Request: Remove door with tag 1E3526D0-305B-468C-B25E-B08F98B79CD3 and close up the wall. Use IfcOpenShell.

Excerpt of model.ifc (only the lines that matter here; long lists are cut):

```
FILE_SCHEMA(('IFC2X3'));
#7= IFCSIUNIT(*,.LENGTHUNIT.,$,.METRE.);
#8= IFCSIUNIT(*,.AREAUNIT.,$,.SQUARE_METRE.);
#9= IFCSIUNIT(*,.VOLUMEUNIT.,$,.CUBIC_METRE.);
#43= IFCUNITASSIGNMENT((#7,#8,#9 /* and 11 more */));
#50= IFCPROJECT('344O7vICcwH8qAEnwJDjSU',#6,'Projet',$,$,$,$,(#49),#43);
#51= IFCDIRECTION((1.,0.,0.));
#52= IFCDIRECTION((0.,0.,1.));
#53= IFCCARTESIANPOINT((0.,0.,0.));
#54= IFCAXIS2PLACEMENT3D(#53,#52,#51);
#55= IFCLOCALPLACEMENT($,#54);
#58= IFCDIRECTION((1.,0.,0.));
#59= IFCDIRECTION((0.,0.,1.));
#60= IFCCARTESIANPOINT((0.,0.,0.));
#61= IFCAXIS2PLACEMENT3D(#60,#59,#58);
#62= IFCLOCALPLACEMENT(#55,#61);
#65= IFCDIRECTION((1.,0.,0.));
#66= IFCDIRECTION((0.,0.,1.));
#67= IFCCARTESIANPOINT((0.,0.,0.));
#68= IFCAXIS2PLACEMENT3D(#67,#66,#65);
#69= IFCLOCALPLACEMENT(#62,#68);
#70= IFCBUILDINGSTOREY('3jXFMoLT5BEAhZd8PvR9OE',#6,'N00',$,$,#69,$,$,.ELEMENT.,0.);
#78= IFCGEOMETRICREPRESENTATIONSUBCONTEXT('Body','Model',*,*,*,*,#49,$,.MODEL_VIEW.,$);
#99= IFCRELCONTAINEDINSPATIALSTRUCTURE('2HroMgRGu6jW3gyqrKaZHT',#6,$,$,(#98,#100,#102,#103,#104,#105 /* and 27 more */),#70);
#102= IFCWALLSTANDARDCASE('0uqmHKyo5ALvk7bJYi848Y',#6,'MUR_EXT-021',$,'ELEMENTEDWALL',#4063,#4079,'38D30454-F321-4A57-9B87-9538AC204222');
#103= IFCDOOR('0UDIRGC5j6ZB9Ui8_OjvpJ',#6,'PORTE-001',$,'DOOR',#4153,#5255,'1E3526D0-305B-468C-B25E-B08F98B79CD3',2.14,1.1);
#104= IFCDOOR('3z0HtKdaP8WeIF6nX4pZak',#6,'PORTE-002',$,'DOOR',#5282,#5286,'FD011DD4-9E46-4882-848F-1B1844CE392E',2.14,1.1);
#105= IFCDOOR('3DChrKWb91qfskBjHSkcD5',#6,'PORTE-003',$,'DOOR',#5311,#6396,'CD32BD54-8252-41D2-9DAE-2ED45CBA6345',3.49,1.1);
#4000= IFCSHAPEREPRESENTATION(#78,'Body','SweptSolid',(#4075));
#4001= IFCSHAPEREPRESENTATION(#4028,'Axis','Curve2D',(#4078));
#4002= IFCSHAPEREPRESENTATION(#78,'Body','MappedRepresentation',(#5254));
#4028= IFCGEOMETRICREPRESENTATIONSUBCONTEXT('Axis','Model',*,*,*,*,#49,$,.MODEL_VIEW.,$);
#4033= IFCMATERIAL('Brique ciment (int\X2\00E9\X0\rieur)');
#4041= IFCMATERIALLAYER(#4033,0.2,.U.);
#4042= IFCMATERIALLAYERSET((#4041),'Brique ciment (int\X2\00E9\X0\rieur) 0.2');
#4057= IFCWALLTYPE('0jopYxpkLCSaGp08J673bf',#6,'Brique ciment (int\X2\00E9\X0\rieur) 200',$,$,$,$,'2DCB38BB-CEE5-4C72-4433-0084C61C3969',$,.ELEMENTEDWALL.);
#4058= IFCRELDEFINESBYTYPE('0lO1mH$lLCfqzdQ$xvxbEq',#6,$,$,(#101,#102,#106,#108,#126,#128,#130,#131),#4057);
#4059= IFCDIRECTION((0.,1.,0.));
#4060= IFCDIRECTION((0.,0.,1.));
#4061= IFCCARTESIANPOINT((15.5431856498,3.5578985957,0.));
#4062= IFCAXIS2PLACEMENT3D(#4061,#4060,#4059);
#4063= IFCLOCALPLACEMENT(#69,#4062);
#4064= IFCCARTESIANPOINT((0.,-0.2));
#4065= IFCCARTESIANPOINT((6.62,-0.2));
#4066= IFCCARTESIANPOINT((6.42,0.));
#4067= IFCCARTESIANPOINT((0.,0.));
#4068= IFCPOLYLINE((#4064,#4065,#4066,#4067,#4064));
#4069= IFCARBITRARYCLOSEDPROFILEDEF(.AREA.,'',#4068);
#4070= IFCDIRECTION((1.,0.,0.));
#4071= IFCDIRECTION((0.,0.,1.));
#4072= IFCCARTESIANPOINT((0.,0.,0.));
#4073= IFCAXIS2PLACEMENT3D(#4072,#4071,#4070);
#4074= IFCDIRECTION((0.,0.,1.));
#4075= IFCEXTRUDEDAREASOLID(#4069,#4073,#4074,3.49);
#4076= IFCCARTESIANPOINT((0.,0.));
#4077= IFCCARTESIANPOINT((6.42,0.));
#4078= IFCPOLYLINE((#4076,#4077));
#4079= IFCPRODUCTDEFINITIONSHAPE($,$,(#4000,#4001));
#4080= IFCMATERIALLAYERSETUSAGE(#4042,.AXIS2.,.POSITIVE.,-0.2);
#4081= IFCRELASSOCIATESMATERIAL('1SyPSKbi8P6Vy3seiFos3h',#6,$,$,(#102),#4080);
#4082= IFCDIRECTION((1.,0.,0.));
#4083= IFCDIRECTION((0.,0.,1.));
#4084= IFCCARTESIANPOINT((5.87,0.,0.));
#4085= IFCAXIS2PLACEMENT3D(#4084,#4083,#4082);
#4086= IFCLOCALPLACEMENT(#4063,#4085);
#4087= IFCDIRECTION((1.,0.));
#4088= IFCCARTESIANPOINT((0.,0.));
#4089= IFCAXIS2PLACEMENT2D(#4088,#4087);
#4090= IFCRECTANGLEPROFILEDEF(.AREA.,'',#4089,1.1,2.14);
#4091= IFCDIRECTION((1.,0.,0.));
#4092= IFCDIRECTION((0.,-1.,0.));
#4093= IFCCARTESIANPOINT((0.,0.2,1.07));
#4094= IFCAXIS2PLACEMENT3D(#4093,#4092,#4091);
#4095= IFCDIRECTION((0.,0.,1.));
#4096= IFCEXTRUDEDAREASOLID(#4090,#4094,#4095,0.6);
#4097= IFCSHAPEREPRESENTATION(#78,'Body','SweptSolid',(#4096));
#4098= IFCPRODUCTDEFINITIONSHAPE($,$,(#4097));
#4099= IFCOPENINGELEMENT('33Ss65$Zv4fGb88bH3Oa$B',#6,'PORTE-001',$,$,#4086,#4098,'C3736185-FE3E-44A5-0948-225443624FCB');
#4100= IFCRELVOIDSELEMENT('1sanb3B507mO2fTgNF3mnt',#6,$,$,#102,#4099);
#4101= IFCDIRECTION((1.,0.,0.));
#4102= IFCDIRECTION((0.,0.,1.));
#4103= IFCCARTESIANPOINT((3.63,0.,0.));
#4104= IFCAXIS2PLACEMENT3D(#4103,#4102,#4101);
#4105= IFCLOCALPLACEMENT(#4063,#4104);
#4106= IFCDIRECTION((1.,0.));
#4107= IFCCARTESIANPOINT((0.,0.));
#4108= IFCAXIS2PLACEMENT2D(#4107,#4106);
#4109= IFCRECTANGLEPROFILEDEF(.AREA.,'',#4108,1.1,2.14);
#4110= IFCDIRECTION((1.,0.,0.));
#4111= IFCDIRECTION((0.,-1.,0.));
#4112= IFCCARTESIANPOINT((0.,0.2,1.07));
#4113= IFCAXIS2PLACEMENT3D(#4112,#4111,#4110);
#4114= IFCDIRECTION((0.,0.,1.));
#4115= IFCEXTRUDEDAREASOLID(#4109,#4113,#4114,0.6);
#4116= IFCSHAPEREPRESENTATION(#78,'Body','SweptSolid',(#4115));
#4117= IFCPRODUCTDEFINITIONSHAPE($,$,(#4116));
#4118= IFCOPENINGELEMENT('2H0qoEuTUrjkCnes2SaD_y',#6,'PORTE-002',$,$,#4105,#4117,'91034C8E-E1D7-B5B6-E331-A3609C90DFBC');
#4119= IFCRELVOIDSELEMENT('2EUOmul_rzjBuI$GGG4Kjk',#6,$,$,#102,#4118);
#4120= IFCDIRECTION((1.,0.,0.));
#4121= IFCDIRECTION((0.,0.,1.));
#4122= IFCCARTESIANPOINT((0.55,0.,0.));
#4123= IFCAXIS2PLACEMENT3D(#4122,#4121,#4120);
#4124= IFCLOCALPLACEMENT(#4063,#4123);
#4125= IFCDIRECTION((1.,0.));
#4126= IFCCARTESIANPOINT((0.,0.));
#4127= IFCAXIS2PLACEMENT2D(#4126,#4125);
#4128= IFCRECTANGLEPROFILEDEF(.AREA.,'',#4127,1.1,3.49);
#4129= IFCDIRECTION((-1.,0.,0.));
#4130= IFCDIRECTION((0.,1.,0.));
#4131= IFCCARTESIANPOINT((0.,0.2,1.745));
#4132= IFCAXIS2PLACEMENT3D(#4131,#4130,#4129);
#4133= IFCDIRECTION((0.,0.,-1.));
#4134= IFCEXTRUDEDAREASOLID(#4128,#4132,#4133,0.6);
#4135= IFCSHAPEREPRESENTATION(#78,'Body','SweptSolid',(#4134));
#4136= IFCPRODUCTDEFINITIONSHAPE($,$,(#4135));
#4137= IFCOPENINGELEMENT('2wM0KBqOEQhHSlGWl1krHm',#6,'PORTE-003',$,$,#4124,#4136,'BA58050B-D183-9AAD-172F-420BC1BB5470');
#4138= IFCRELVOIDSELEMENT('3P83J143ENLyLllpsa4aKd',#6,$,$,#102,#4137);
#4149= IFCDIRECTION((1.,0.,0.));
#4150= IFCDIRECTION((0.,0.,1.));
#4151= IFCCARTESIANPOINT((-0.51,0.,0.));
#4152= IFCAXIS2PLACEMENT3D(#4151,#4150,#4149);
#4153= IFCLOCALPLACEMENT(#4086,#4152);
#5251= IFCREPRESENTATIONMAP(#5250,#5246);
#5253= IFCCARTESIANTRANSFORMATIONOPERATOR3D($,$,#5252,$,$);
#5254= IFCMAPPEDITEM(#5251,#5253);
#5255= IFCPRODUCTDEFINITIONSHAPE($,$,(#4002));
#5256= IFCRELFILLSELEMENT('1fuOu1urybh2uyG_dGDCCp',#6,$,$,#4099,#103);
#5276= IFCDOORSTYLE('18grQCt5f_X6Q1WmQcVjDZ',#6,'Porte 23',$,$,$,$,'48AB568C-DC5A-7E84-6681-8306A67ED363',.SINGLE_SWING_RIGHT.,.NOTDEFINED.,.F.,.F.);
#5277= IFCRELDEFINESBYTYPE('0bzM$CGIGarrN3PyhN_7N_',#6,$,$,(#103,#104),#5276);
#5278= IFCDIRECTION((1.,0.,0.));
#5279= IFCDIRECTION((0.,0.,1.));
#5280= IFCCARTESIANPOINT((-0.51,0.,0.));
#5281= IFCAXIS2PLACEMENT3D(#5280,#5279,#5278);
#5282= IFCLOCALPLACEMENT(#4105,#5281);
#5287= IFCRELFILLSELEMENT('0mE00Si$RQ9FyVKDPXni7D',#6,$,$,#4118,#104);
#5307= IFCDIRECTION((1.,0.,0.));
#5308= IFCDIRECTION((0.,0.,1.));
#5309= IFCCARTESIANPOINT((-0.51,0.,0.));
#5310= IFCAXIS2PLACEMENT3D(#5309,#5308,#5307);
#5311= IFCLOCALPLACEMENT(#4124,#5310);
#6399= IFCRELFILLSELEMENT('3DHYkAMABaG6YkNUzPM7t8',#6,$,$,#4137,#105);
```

```python
import ifcopenshell
import ifcopenshell.api.feature
import ifcopenshell.api.root
import ifcopenshell.geom
import ifcopenshell.util.shape

model = ifcopenshell.open("model.ifc")
settings = ifcopenshell.geom.settings()


def volume(element):
    """Net volume in cubic metres, openings subtracted."""
    shape = ifcopenshell.geom.create_shape(settings, element)
    return ifcopenshell.util.shape.get_volume(shape.geometry)


door = model.by_id(103)
opening = door.FillsVoids[0].RelatingOpeningElement
wall = opening.VoidsElements[0].RelatingBuildingElement
before = volume(wall)

ifcopenshell.api.root.remove_product(model, product=door)
ifcopenshell.api.feature.remove_feature(model, feature=opening)

after = volume(wall)

print(f"wall volume {before:.3f} -> {after:.3f} m3")

model.write("model_v2.ifc")
```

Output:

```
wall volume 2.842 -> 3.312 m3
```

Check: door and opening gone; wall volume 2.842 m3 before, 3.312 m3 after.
